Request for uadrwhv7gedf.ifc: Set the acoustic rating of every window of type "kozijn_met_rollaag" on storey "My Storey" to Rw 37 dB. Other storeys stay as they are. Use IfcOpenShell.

First a look at what the model holds.

```python
import ifcopenshell
import ifcopenshell.util.element

model = ifcopenshell.open("uadrwhv7gedf.ifc")
print(model.schema)
storey = next(s for s in model.by_type("IfcBuildingStorey") if s.Name == "My Storey")
windows = [e for e in ifcopenshell.util.element.get_decomposition(storey) if e.is_a("IfcWindow")]
seen = {}
for e in windows:
    element_type = ifcopenshell.util.element.get_type(e)
    key = (element_type.Name if element_type != e and element_type else None, ifcopenshell.util.element.get_pset(e, "Pset_WindowCommon", "AcousticRating"))
    seen[key] = seen.get(key, 0) + 1
for (name, value), count in sorted(seen.items(), key=str):
    print(count, "x", name, "|", value)
```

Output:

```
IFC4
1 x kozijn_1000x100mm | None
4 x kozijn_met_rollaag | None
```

```python
import ifcopenshell
import ifcopenshell.api.pset
import ifcopenshell.util.element

model = ifcopenshell.open("uadrwhv7gedf.ifc")

storey = next(s for s in model.by_type("IfcBuildingStorey") if s.Name == "My Storey")
windows = [e for e in ifcopenshell.util.element.get_decomposition(storey) if e.is_a("IfcWindow")]

count = 0
for e in windows:
    element_type = ifcopenshell.util.element.get_type(e)
    if element_type in (None, e) or element_type.Name != "kozijn_met_rollaag":
        continue
    # add_pset returns the element's existing set when there is one.
    pset = ifcopenshell.api.pset.add_pset(model, product=e, name="Pset_WindowCommon")
    ifcopenshell.api.pset.edit_pset(model, pset=pset, properties={"AcousticRating": "Rw 37 dB"})
    count += 1

print(count, "windows updated")

model.write("uadrwhv7gedf_v2.ifc")
```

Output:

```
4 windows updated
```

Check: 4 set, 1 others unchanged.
